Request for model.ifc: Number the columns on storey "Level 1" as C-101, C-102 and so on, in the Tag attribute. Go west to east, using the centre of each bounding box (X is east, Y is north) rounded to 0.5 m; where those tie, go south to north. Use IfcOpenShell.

First a look at what the model holds.

```python
import ifcopenshell
import ifcopenshell.util.element
import ifcopenshell.util.placement

model = ifcopenshell.open("model.ifc")
print(model.schema)
storey = next(s for s in model.by_type("IfcBuildingStorey") if s.Name == "Level 1")
columns = [e for e in ifcopenshell.util.element.get_decomposition(storey) if e.is_a("IfcColumn")]
for e in sorted(columns, key=lambda e: e.id()):
    origin = ifcopenshell.util.placement.get_local_placement(e.ObjectPlacement)[:3, 3]
    print(e.id(), e.Tag, e.Name, origin.round(2) + 0.0, sep=" | ")
```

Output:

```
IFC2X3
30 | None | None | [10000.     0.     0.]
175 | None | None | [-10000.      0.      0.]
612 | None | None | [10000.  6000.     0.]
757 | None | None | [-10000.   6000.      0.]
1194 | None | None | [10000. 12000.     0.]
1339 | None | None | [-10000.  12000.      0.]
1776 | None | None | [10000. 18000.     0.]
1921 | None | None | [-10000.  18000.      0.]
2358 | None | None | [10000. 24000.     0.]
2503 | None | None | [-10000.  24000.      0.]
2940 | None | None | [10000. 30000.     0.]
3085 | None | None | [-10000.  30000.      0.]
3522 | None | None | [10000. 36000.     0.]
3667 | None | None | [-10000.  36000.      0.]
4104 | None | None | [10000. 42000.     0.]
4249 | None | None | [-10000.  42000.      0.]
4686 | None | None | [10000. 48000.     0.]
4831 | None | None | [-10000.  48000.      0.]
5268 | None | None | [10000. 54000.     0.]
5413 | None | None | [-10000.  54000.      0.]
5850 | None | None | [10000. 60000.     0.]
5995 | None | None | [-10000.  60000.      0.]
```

```python
import ifcopenshell
import ifcopenshell.geom
import ifcopenshell.util.element
import ifcopenshell.util.shape

model = ifcopenshell.open("model.ifc")
settings = ifcopenshell.geom.settings()
settings.set("use-world-coords", True)


def centre(element):
    shape = ifcopenshell.geom.create_shape(settings, element)
    return ifcopenshell.util.shape.get_bbox_centroid(shape.geometry)


storey = next(s for s in model.by_type("IfcBuildingStorey") if s.Name == "Level 1")
columns = [e for e in ifcopenshell.util.element.get_decomposition(storey) if e.is_a("IfcColumn")]

# Insertion points can sit at a corner or the storey origin, so sort by the geometry (in metres).
centres = {e: centre(e) for e in columns}
columns.sort(key=lambda e: (round(centres[e][0] / 0.5), centres[e][1]))

for i, e in enumerate(columns, start=1):
    number = f"C-1{i:02d}"
    e.Tag = number
    print(e.id(), number)

model.write("model_rev.ifc")
```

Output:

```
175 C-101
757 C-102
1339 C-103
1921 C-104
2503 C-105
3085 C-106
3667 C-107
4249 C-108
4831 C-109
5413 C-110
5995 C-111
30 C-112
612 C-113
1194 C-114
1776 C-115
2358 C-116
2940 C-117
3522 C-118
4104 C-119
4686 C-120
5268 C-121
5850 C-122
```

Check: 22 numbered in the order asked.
